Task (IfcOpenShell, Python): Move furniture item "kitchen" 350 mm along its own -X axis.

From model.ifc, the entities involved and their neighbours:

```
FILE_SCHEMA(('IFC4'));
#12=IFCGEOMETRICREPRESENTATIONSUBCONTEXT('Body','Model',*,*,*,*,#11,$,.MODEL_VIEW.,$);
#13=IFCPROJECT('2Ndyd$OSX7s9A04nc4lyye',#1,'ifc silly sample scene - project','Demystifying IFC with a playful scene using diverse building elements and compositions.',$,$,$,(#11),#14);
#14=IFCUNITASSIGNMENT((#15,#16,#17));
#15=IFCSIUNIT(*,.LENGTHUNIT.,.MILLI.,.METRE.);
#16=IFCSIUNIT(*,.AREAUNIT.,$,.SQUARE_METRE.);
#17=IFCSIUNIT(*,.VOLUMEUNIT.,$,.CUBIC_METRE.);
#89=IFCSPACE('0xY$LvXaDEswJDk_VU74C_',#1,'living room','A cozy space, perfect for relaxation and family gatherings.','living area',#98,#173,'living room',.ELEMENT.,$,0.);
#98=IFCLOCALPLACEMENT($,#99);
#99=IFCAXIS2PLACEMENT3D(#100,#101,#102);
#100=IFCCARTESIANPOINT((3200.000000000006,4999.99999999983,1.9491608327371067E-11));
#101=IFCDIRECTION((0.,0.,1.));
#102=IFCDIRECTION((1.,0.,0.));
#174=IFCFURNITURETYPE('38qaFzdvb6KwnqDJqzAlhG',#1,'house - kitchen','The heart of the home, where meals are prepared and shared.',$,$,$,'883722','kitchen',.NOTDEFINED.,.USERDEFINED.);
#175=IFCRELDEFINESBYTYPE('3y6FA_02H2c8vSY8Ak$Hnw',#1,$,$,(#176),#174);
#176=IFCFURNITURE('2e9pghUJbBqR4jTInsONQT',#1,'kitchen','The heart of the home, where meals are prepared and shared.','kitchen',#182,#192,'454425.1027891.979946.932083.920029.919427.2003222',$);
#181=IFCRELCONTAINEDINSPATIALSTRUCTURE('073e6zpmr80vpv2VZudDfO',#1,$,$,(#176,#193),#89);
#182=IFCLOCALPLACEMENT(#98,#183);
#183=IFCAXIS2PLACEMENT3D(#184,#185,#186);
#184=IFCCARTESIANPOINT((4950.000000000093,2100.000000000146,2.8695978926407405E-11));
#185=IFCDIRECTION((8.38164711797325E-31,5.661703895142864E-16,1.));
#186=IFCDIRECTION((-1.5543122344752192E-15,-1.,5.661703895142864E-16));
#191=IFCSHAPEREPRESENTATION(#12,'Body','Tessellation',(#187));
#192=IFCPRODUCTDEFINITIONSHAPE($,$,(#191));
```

```python
import ifcopenshell
import ifcopenshell.api.geometry
import ifcopenshell.util.placement

model = ifcopenshell.open("model.ifc")

item = model.by_guid("2e9pghUJbBqR4jTInsONQT")
matrix = ifcopenshell.util.placement.get_local_placement(item.ObjectPlacement)
matrix[:3, 3] -= matrix[:3, 0] * 350.0
ifcopenshell.api.geometry.edit_object_placement(model, product=item, matrix=matrix, is_si=False)

print(ifcopenshell.util.placement.get_local_placement(item.ObjectPlacement).round(3) + 0.0)

model.write("model_edited.ifc")
```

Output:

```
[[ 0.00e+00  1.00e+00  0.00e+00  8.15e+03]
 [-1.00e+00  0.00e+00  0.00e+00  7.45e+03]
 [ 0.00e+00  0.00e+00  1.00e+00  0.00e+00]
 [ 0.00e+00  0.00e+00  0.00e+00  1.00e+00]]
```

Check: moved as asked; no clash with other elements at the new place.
